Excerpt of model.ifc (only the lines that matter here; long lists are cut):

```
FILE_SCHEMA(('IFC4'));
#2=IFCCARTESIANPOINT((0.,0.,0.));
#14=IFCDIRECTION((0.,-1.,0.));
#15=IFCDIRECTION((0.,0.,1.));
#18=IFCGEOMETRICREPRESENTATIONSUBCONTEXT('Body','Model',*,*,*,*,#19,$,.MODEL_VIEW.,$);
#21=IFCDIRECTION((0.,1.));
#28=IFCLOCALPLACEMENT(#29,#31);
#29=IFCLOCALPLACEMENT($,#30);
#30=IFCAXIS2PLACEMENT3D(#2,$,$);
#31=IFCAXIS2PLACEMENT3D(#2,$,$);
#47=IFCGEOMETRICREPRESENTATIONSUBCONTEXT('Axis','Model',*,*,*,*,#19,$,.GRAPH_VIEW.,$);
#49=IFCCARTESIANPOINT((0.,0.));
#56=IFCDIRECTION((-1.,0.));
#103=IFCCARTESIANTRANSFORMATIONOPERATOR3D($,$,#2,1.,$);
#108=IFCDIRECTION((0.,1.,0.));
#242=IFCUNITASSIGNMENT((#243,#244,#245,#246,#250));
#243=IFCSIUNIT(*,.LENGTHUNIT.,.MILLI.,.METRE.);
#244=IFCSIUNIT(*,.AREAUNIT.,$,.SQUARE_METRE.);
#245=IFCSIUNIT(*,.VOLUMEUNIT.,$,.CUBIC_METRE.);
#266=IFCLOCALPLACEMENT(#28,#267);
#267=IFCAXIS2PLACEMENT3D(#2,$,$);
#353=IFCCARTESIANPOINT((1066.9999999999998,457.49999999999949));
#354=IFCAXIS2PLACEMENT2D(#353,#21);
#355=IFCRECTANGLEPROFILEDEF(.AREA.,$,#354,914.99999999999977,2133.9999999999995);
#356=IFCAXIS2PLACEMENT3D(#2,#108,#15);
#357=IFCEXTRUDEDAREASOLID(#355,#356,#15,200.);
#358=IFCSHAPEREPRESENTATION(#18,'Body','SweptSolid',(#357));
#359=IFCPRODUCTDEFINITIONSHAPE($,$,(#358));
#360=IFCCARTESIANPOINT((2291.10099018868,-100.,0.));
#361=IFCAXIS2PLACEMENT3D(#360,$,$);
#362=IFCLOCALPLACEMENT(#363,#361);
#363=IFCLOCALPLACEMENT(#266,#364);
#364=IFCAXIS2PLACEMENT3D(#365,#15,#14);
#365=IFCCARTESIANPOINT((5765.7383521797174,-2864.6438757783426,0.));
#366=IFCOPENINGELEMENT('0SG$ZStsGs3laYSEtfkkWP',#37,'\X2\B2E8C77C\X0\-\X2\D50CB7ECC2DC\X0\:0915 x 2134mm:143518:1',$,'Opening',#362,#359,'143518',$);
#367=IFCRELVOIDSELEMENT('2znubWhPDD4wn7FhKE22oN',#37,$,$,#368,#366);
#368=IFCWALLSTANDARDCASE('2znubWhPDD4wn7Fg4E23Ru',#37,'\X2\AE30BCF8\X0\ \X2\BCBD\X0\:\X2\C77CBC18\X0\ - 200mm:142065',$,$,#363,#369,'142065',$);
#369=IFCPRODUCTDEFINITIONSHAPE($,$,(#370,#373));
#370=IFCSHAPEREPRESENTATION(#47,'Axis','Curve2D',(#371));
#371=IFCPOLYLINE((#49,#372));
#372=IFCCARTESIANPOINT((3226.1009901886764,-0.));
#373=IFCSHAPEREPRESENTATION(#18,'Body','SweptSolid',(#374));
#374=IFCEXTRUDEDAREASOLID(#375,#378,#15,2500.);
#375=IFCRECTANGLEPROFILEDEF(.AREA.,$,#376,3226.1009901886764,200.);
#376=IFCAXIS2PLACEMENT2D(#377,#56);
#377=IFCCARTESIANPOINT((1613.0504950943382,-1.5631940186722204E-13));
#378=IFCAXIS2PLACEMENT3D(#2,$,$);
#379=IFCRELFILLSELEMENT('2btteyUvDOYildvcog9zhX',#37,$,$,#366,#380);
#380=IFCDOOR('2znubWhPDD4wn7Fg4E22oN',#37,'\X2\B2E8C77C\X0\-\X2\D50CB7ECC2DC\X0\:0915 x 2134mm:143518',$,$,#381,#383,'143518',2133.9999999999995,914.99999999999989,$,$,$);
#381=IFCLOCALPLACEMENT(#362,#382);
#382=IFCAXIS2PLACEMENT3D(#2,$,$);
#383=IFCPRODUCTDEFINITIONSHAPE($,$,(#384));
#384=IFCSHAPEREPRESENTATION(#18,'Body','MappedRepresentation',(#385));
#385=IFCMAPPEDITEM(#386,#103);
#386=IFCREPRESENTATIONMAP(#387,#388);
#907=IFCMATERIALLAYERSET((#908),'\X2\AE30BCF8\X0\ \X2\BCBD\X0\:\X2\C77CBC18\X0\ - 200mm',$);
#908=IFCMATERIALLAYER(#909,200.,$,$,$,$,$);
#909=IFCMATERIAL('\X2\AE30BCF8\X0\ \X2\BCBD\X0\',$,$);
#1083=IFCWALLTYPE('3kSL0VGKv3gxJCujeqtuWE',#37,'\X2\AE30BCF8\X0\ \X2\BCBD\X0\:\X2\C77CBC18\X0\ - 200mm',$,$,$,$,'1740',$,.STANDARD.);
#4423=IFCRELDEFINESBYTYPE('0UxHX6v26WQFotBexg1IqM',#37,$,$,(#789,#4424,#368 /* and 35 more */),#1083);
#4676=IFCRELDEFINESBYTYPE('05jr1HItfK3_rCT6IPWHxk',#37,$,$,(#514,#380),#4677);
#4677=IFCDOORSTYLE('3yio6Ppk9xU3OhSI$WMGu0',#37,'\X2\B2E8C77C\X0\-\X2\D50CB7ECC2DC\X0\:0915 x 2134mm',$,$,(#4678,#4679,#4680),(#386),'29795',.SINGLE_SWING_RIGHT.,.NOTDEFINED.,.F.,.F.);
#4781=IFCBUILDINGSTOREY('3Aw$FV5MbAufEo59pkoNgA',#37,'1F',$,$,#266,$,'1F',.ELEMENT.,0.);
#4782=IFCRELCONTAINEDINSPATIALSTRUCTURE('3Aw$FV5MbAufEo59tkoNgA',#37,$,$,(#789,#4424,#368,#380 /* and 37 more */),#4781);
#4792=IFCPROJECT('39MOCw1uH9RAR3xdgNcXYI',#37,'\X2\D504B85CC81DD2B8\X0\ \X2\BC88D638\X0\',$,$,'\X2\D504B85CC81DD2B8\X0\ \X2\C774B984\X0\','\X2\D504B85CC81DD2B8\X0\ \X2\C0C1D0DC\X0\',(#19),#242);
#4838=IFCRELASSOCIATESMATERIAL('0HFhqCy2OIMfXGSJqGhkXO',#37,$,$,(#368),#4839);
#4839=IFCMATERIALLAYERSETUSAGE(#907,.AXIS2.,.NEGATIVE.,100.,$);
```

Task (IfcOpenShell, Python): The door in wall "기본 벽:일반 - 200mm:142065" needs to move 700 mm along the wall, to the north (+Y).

```python
import ifcopenshell
import ifcopenshell.api.geometry
import ifcopenshell.util.placement
import ifcopenshell.util.unit

model = ifcopenshell.open("model.ifc")
unit_scale = ifcopenshell.util.unit.calculate_unit_scale(model)

door = model.by_id(380)
opening = door.FillsVoids[0].RelatingOpeningElement
wall = opening.VoidsElements[0].RelatingBuildingElement

wall_matrix = ifcopenshell.util.placement.get_local_placement(wall.ObjectPlacement)
shift = wall_matrix[:3, 0] * -0.7 / unit_scale
before = ifcopenshell.util.placement.get_local_placement(door.ObjectPlacement)[:3, 3].copy()

# The door is placed relative to its opening, so it follows when the opening moves.
matrix = ifcopenshell.util.placement.get_local_placement(opening.ObjectPlacement)
matrix[:3, 3] += shift
ifcopenshell.api.geometry.edit_object_placement(
    model, product=opening, matrix=matrix, is_si=False, should_transform_children=True
)

after = ifcopenshell.util.placement.get_local_placement(door.ObjectPlacement)[:3, 3]
print("door moved by", (after - before).round(3) + 0.0)

model.write("model_rev.ifc")
```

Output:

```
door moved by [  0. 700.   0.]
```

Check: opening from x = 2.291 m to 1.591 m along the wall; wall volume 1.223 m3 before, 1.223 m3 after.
